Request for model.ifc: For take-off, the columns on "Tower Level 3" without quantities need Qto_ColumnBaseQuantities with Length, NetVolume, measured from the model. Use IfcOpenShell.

First a look at what the model holds.

```python
import ifcopenshell
import ifcopenshell.util.element
import ifcopenshell.util.unit

model = ifcopenshell.open("model.ifc")
print(model.schema)
for unit_type in ("LENGTHUNIT", "AREAUNIT", "VOLUMEUNIT"):
    print(unit_type, ifcopenshell.util.unit.calculate_unit_scale(model, unit_type))
storey = next(s for s in model.by_type("IfcBuildingStorey") if s.Name == "Tower Level 3")
columns = [e for e in ifcopenshell.util.element.get_decomposition(storey) if e.is_a("IfcColumn")]
for e in sorted(columns, key=lambda e: e.id()):
    print(e.id(), e.is_a(), e.Name, list(ifcopenshell.util.element.get_psets(e, qtos_only=True)), sep=" | ")
```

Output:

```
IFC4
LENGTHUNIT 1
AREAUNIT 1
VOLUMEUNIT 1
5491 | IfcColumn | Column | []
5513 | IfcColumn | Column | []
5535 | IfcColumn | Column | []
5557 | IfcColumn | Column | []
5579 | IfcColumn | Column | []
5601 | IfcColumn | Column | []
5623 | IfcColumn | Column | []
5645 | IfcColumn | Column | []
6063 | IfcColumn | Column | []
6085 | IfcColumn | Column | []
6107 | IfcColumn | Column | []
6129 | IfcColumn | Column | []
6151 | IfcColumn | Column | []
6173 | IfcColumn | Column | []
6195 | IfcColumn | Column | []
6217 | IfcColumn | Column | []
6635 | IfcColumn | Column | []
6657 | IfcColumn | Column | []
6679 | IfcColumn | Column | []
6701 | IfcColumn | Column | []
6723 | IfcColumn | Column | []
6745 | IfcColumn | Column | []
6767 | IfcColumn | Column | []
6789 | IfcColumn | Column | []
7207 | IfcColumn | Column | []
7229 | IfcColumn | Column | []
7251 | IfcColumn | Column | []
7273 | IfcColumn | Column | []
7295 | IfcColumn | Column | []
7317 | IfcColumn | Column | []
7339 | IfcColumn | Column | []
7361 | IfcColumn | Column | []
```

```python
import ifcopenshell
import ifcopenshell.api.pset
import ifcopenshell.geom
import ifcopenshell.util.element
import ifcopenshell.util.shape
import ifcopenshell.util.unit

model = ifcopenshell.open("model.ifc")
unit_scale = ifcopenshell.util.unit.calculate_unit_scale(model)
volume_scale = ifcopenshell.util.unit.calculate_unit_scale(model, "VOLUMEUNIT")
settings = ifcopenshell.geom.settings()

storey = next(s for s in model.by_type("IfcBuildingStorey") if s.Name == "Tower Level 3")
columns = [e for e in ifcopenshell.util.element.get_decomposition(storey) if e.is_a("IfcColumn")]

for e in sorted(columns, key=lambda e: e.id()):
    if ifcopenshell.util.element.get_psets(e, qtos_only=True, should_inherit=False):
        continue
    # Geometry comes back in metres, in the element's own axes.
    shape = ifcopenshell.geom.create_shape(settings, e)
    values = {
        "Length": ifcopenshell.util.shape.get_z(shape.geometry) / unit_scale,
        "NetVolume": ifcopenshell.util.shape.get_volume(shape.geometry) / volume_scale,
    }
    qto = ifcopenshell.api.pset.add_qto(model, product=e, name="Qto_ColumnBaseQuantities")
    ifcopenshell.api.pset.edit_qto(model, qto=qto, properties=values)
    print(e.id(), {k: round(v, 3) for k, v in values.items()})

model.write("model_v2.ifc")
```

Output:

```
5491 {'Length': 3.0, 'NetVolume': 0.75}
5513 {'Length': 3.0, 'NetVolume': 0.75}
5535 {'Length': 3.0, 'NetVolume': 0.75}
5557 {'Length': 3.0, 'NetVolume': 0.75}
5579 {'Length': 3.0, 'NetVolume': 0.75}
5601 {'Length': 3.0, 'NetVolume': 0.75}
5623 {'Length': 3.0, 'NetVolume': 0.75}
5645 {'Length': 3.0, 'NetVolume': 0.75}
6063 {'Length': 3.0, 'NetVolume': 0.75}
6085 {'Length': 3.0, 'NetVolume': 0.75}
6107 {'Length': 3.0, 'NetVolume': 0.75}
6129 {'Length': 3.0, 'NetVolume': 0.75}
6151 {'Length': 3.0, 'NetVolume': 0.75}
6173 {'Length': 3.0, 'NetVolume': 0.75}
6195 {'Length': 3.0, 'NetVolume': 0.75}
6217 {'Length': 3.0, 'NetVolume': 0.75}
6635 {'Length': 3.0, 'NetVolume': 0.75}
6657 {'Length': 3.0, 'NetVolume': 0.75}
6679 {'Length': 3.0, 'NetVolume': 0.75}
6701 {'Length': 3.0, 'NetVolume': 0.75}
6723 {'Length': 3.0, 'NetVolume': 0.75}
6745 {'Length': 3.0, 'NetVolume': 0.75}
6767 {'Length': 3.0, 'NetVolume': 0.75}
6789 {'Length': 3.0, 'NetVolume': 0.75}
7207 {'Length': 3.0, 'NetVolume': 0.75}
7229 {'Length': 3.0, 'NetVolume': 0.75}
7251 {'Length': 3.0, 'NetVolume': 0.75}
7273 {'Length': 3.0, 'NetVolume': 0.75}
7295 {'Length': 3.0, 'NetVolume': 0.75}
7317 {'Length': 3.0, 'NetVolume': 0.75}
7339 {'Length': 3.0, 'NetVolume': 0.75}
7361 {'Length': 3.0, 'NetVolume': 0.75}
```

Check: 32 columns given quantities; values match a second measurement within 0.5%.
